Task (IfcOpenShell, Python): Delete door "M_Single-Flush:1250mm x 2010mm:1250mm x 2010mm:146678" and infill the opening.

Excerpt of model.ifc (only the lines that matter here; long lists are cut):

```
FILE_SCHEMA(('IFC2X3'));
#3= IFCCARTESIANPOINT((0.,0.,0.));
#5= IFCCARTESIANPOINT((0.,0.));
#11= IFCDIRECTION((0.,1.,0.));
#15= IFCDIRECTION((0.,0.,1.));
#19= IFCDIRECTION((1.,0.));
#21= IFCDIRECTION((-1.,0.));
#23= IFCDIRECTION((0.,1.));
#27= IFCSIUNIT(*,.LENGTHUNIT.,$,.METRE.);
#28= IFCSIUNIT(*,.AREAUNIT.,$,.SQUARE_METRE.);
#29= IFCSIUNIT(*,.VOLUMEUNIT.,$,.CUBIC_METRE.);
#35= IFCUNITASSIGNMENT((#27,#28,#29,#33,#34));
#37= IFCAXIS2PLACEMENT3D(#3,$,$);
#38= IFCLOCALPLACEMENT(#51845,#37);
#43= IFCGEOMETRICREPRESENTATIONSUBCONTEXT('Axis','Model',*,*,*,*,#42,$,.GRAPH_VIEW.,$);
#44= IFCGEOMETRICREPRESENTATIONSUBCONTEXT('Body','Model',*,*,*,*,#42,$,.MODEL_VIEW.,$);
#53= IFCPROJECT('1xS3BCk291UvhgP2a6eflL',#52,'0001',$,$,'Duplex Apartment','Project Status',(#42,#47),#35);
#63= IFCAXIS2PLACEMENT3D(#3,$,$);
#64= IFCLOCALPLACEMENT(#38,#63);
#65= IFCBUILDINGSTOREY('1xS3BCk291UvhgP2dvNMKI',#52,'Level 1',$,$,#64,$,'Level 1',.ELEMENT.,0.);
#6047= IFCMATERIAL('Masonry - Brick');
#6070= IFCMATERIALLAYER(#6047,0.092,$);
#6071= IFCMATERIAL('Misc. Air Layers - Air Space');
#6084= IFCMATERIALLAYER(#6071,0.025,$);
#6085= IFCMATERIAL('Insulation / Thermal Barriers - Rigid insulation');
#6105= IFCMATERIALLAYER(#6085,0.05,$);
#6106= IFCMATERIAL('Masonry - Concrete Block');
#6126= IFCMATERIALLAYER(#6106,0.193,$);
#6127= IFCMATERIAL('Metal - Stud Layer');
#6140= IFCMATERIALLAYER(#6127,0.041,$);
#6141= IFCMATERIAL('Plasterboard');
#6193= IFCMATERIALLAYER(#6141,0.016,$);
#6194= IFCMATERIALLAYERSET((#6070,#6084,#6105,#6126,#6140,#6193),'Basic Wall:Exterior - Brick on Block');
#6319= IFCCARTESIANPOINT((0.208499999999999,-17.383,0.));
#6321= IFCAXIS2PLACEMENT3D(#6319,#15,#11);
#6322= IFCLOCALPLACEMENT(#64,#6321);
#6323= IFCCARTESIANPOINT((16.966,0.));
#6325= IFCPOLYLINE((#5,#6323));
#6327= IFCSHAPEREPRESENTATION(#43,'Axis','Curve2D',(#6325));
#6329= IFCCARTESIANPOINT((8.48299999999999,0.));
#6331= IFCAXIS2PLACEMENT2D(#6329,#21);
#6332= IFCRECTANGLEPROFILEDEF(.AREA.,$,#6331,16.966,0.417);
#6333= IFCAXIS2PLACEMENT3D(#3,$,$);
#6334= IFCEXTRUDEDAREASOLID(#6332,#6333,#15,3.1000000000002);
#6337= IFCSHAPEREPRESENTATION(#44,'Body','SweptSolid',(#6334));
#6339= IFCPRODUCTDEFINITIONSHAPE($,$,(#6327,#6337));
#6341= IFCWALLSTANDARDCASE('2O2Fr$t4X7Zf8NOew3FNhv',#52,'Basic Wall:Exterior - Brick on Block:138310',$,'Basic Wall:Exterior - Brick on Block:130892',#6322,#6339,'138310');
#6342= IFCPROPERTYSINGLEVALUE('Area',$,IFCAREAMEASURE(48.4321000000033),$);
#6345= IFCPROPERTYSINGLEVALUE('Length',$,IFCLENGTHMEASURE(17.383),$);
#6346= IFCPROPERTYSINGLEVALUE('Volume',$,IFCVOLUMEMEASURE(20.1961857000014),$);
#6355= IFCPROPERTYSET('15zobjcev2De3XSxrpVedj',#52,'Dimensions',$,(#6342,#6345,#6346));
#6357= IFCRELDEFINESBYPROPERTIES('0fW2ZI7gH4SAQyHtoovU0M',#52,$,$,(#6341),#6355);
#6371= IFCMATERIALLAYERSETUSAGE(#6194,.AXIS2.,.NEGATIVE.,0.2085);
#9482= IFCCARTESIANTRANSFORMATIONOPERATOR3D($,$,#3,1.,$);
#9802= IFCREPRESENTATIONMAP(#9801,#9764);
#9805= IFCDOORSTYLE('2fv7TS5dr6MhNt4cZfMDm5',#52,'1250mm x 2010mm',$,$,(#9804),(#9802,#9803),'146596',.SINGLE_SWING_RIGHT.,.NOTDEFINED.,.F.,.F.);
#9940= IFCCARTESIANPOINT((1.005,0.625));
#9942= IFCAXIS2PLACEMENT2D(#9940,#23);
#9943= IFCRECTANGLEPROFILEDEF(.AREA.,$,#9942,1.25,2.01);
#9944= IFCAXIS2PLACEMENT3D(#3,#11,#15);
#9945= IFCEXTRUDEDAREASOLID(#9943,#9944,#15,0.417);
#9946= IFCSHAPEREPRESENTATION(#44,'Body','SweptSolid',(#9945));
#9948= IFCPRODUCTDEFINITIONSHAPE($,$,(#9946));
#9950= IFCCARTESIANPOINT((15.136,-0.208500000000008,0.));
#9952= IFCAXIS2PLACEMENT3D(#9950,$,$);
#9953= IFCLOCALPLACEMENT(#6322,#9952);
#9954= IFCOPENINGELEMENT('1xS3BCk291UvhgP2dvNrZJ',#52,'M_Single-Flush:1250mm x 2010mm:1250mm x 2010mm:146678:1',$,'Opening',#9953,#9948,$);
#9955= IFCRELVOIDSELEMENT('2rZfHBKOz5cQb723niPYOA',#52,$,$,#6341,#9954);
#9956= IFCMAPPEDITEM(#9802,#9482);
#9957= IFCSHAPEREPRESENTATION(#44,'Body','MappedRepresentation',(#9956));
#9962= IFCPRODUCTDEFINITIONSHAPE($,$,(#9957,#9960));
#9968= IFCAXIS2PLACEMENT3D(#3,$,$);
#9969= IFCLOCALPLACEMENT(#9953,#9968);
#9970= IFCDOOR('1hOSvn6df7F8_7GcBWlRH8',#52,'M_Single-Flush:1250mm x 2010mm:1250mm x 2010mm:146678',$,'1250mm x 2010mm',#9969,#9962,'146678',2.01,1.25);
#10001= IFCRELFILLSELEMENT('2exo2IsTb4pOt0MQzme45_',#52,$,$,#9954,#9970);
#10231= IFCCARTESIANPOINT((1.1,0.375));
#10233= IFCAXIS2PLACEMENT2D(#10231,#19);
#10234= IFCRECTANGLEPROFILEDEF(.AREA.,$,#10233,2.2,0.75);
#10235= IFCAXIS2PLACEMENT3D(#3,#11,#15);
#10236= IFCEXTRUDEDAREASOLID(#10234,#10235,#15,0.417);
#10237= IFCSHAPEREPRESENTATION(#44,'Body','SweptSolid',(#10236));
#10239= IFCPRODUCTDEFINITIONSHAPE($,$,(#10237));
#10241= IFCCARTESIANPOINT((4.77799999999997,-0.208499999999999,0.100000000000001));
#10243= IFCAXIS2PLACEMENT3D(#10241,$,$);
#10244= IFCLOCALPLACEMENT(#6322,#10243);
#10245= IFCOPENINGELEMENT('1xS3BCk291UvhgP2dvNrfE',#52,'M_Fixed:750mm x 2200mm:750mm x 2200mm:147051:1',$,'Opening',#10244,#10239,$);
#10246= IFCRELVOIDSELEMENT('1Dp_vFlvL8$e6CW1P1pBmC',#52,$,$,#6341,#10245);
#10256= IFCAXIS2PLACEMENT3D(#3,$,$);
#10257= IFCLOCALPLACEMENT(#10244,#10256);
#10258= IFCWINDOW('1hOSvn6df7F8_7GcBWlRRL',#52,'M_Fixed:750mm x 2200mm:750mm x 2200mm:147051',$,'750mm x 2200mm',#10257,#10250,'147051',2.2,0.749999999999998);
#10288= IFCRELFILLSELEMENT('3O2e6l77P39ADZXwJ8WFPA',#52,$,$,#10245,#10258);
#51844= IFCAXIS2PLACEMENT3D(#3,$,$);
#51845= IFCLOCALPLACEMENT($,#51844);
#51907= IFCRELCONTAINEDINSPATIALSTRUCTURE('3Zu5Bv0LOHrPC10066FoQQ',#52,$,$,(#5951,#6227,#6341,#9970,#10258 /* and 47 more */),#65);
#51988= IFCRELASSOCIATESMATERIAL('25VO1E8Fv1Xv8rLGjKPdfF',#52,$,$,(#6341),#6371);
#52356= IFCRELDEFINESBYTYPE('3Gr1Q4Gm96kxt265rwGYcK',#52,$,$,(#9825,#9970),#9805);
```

```python
import ifcopenshell
import ifcopenshell.api.feature
import ifcopenshell.api.pset
import ifcopenshell.api.root
import ifcopenshell.geom
import ifcopenshell.util.element
import ifcopenshell.util.shape
import ifcopenshell.util.unit

model = ifcopenshell.open("model.ifc")
area_scale = ifcopenshell.util.unit.calculate_unit_scale(model, "AREAUNIT")
volume_scale = ifcopenshell.util.unit.calculate_unit_scale(model, "VOLUMEUNIT")
settings = ifcopenshell.geom.settings()


def volume(element):
    """Net volume in cubic metres, openings subtracted."""
    shape = ifcopenshell.geom.create_shape(settings, element)
    return ifcopenshell.util.shape.get_volume(shape.geometry)


door = model.by_guid("1hOSvn6df7F8_7GcBWlRH8")
opening = door.FillsVoids[0].RelatingOpeningElement
wall = opening.VoidsElements[0].RelatingBuildingElement
before = volume(wall)

ifcopenshell.api.root.remove_product(model, product=door)
ifcopenshell.api.feature.remove_feature(model, feature=opening)

after = volume(wall)
thickness = 0.417  # wall thickness in metres

# Update the wall's stored quantities.
pset = model.by_id(ifcopenshell.util.element.get_pset(wall, "Dimensions", should_inherit=False)["id"])
ifcopenshell.api.pset.edit_pset(model, pset=pset, properties={
    "Area": model.create_entity("IfcAreaMeasure", after / thickness / area_scale),
    "Volume": model.create_entity("IfcVolumeMeasure", after / volume_scale),
})

print(f"wall volume {before:.3f} -> {after:.3f} m3")

model.write("model_v2.ifc")
```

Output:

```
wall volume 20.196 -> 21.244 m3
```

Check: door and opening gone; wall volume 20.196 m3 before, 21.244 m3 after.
